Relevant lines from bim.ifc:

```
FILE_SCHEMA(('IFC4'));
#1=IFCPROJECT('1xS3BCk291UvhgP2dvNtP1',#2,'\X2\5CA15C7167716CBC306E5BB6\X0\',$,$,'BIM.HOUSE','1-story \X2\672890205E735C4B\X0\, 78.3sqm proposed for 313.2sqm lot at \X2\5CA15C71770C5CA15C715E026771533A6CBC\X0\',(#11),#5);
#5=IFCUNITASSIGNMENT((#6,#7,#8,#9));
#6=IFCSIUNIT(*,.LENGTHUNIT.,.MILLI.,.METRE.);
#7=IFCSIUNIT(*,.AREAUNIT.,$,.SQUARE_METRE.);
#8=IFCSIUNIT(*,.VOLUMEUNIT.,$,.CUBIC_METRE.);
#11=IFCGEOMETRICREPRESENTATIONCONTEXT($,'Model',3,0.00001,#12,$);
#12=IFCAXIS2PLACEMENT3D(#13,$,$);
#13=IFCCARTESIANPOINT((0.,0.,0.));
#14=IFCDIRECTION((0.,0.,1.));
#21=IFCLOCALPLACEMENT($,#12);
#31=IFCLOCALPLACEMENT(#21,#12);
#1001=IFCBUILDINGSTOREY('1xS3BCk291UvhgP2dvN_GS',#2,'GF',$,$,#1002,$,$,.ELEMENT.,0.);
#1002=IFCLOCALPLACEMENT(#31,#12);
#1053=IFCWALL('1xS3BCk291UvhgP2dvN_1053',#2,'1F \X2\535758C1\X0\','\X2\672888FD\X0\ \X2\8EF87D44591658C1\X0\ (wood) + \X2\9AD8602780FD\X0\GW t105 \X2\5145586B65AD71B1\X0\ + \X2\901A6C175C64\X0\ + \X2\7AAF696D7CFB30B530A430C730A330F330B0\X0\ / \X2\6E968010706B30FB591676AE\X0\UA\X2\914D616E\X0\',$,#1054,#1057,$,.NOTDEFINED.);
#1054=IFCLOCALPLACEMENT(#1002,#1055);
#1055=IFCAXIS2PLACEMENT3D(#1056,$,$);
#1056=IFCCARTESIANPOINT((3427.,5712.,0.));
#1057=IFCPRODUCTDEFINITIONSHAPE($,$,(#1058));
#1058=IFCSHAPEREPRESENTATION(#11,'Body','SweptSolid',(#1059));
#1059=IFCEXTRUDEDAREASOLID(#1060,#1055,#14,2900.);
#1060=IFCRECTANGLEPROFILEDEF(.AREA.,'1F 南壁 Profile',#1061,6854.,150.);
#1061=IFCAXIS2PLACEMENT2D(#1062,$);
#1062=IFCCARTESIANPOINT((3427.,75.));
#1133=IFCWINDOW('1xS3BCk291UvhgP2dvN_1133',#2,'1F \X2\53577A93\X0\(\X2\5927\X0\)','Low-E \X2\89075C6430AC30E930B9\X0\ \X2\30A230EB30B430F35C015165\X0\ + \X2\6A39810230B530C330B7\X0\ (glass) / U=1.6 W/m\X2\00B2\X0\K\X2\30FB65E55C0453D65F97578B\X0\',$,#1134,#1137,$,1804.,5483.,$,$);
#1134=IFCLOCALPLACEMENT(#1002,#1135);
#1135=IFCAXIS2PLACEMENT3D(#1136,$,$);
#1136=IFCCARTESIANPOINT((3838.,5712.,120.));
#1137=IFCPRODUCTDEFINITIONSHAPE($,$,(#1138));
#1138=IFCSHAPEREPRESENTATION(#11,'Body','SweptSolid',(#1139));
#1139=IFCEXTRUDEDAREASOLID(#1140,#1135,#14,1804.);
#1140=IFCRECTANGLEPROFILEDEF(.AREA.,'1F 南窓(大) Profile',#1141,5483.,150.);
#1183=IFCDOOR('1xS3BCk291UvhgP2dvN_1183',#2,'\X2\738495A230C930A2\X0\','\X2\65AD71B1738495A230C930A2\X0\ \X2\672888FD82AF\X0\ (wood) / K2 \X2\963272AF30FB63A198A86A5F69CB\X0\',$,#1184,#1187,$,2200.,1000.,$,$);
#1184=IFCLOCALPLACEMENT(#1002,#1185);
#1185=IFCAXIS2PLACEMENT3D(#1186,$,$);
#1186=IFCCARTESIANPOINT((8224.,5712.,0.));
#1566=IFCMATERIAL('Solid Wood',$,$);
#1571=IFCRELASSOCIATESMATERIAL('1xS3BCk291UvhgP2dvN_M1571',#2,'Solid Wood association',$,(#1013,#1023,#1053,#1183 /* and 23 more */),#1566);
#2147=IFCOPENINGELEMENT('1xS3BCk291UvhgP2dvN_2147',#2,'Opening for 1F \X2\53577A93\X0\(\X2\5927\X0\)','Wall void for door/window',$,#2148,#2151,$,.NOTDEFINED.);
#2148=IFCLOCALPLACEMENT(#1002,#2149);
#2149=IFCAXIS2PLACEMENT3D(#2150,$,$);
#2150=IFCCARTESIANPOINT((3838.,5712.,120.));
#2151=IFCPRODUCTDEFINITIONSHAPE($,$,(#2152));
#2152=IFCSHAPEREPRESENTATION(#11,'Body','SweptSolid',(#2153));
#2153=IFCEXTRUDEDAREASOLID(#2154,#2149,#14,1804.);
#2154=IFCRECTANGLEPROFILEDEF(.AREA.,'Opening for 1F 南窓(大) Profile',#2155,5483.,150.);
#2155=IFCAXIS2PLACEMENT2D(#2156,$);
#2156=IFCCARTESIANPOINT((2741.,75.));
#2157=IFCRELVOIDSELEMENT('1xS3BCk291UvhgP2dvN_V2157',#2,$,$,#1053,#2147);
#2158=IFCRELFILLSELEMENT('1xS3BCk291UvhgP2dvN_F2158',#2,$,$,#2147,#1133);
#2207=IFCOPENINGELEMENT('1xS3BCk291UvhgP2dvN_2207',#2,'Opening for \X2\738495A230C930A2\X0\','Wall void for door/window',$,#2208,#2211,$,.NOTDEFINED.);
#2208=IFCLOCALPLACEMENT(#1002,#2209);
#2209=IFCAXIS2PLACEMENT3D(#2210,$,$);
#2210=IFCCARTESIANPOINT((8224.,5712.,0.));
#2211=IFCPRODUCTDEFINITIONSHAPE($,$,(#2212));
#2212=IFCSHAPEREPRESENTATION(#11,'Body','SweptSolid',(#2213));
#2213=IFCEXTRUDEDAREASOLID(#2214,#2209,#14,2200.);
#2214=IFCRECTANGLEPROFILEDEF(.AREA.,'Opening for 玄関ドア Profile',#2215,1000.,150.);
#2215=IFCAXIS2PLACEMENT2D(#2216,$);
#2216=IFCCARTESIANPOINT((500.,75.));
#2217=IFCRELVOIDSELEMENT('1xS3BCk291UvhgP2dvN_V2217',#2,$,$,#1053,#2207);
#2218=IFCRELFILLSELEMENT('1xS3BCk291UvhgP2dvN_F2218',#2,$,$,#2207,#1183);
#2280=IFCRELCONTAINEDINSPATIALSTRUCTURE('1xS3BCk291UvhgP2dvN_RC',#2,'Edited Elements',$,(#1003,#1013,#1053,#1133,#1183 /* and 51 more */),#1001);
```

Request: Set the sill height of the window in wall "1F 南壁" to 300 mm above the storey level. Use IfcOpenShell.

```python
import numpy as np
import ifcopenshell
import ifcopenshell.api.geometry
import ifcopenshell.geom
import ifcopenshell.util.element
import ifcopenshell.util.placement
import ifcopenshell.util.shape
import ifcopenshell.util.unit

model = ifcopenshell.open("bim.ifc")
unit_scale = ifcopenshell.util.unit.calculate_unit_scale(model)

window = model.by_guid("1xS3BCk291UvhgP2dvN_1133")
opening = window.FillsVoids[0].RelatingOpeningElement
storey = ifcopenshell.util.element.get_container(window, ifc_class="IfcBuildingStorey")
level = ifcopenshell.util.placement.get_local_placement(storey.ObjectPlacement)[2, 3]

# The opening's origin need not be at the sill, so measure its lowest point.
shape = ifcopenshell.geom.create_shape(ifcopenshell.geom.settings(), opening)
bottom = ifcopenshell.util.shape.get_shape_bottom_elevation(shape, shape.geometry) / unit_scale
dz = level + 300.0 - bottom

shift = np.array([0.0, 0.0, dz])
# The window is not placed relative to its opening, so move both.
for product in (opening, window):
    matrix = ifcopenshell.util.placement.get_local_placement(product.ObjectPlacement)
    matrix[:3, 3] += shift
    ifcopenshell.api.geometry.edit_object_placement(model, product=product, matrix=matrix, is_si=False)

print(f"moved by {dz * unit_scale:+.3f} m")

model.write("bim_rev.ifc")
```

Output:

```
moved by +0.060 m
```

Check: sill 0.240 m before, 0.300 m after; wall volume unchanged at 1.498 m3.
